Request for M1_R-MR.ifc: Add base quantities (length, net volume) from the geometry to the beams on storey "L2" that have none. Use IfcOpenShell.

First a look at what the model holds.

```python
import ifcopenshell
import ifcopenshell.util.element
import ifcopenshell.util.unit

model = ifcopenshell.open("M1_R-MR.ifc")
print(model.schema)
for unit_type in ("LENGTHUNIT", "AREAUNIT", "VOLUMEUNIT"):
    print(unit_type, ifcopenshell.util.unit.calculate_unit_scale(model, unit_type))
storey = next(s for s in model.by_type("IfcBuildingStorey") if s.Name == "L2")
beams = [e for e in ifcopenshell.util.element.get_decomposition(storey) if e.is_a("IfcBeam")]
for e in sorted(beams, key=lambda e: e.id()):
    print(e.id(), e.is_a(), e.Name, list(ifcopenshell.util.element.get_psets(e, qtos_only=True)), sep=" | ")
```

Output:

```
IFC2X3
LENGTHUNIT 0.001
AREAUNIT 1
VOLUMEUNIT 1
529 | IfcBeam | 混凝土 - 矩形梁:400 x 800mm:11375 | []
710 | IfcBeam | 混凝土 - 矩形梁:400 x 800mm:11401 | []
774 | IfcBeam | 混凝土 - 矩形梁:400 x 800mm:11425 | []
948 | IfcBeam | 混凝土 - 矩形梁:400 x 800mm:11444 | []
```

```python
import ifcopenshell
import ifcopenshell.api.pset
import ifcopenshell.geom
import ifcopenshell.util.element
import ifcopenshell.util.shape
import ifcopenshell.util.unit

model = ifcopenshell.open("M1_R-MR.ifc")
unit_scale = ifcopenshell.util.unit.calculate_unit_scale(model)
volume_scale = ifcopenshell.util.unit.calculate_unit_scale(model, "VOLUMEUNIT")
settings = ifcopenshell.geom.settings()

storey = next(s for s in model.by_type("IfcBuildingStorey") if s.Name == "L2")
beams = [e for e in ifcopenshell.util.element.get_decomposition(storey) if e.is_a("IfcBeam")]

for e in sorted(beams, key=lambda e: e.id()):
    if ifcopenshell.util.element.get_psets(e, qtos_only=True, should_inherit=False):
        continue
    # Geometry comes back in metres, in the element's own axes.
    shape = ifcopenshell.geom.create_shape(settings, e)
    values = {
        "Length": ifcopenshell.util.shape.get_max_xyz(shape.geometry) / unit_scale,
        "NetVolume": ifcopenshell.util.shape.get_volume(shape.geometry) / volume_scale,
    }
    qto = ifcopenshell.api.pset.add_qto(model, product=e, name="BaseQuantities")
    ifcopenshell.api.pset.edit_qto(model, qto=qto, properties=values)
    print(e.id(), {k: round(v, 3) for k, v in values.items()})

model.write("M1_R-MR_rev.ifc")
```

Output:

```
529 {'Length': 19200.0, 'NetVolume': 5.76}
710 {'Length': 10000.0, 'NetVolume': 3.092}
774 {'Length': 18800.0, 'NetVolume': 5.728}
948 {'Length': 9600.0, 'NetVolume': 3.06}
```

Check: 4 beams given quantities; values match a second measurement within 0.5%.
